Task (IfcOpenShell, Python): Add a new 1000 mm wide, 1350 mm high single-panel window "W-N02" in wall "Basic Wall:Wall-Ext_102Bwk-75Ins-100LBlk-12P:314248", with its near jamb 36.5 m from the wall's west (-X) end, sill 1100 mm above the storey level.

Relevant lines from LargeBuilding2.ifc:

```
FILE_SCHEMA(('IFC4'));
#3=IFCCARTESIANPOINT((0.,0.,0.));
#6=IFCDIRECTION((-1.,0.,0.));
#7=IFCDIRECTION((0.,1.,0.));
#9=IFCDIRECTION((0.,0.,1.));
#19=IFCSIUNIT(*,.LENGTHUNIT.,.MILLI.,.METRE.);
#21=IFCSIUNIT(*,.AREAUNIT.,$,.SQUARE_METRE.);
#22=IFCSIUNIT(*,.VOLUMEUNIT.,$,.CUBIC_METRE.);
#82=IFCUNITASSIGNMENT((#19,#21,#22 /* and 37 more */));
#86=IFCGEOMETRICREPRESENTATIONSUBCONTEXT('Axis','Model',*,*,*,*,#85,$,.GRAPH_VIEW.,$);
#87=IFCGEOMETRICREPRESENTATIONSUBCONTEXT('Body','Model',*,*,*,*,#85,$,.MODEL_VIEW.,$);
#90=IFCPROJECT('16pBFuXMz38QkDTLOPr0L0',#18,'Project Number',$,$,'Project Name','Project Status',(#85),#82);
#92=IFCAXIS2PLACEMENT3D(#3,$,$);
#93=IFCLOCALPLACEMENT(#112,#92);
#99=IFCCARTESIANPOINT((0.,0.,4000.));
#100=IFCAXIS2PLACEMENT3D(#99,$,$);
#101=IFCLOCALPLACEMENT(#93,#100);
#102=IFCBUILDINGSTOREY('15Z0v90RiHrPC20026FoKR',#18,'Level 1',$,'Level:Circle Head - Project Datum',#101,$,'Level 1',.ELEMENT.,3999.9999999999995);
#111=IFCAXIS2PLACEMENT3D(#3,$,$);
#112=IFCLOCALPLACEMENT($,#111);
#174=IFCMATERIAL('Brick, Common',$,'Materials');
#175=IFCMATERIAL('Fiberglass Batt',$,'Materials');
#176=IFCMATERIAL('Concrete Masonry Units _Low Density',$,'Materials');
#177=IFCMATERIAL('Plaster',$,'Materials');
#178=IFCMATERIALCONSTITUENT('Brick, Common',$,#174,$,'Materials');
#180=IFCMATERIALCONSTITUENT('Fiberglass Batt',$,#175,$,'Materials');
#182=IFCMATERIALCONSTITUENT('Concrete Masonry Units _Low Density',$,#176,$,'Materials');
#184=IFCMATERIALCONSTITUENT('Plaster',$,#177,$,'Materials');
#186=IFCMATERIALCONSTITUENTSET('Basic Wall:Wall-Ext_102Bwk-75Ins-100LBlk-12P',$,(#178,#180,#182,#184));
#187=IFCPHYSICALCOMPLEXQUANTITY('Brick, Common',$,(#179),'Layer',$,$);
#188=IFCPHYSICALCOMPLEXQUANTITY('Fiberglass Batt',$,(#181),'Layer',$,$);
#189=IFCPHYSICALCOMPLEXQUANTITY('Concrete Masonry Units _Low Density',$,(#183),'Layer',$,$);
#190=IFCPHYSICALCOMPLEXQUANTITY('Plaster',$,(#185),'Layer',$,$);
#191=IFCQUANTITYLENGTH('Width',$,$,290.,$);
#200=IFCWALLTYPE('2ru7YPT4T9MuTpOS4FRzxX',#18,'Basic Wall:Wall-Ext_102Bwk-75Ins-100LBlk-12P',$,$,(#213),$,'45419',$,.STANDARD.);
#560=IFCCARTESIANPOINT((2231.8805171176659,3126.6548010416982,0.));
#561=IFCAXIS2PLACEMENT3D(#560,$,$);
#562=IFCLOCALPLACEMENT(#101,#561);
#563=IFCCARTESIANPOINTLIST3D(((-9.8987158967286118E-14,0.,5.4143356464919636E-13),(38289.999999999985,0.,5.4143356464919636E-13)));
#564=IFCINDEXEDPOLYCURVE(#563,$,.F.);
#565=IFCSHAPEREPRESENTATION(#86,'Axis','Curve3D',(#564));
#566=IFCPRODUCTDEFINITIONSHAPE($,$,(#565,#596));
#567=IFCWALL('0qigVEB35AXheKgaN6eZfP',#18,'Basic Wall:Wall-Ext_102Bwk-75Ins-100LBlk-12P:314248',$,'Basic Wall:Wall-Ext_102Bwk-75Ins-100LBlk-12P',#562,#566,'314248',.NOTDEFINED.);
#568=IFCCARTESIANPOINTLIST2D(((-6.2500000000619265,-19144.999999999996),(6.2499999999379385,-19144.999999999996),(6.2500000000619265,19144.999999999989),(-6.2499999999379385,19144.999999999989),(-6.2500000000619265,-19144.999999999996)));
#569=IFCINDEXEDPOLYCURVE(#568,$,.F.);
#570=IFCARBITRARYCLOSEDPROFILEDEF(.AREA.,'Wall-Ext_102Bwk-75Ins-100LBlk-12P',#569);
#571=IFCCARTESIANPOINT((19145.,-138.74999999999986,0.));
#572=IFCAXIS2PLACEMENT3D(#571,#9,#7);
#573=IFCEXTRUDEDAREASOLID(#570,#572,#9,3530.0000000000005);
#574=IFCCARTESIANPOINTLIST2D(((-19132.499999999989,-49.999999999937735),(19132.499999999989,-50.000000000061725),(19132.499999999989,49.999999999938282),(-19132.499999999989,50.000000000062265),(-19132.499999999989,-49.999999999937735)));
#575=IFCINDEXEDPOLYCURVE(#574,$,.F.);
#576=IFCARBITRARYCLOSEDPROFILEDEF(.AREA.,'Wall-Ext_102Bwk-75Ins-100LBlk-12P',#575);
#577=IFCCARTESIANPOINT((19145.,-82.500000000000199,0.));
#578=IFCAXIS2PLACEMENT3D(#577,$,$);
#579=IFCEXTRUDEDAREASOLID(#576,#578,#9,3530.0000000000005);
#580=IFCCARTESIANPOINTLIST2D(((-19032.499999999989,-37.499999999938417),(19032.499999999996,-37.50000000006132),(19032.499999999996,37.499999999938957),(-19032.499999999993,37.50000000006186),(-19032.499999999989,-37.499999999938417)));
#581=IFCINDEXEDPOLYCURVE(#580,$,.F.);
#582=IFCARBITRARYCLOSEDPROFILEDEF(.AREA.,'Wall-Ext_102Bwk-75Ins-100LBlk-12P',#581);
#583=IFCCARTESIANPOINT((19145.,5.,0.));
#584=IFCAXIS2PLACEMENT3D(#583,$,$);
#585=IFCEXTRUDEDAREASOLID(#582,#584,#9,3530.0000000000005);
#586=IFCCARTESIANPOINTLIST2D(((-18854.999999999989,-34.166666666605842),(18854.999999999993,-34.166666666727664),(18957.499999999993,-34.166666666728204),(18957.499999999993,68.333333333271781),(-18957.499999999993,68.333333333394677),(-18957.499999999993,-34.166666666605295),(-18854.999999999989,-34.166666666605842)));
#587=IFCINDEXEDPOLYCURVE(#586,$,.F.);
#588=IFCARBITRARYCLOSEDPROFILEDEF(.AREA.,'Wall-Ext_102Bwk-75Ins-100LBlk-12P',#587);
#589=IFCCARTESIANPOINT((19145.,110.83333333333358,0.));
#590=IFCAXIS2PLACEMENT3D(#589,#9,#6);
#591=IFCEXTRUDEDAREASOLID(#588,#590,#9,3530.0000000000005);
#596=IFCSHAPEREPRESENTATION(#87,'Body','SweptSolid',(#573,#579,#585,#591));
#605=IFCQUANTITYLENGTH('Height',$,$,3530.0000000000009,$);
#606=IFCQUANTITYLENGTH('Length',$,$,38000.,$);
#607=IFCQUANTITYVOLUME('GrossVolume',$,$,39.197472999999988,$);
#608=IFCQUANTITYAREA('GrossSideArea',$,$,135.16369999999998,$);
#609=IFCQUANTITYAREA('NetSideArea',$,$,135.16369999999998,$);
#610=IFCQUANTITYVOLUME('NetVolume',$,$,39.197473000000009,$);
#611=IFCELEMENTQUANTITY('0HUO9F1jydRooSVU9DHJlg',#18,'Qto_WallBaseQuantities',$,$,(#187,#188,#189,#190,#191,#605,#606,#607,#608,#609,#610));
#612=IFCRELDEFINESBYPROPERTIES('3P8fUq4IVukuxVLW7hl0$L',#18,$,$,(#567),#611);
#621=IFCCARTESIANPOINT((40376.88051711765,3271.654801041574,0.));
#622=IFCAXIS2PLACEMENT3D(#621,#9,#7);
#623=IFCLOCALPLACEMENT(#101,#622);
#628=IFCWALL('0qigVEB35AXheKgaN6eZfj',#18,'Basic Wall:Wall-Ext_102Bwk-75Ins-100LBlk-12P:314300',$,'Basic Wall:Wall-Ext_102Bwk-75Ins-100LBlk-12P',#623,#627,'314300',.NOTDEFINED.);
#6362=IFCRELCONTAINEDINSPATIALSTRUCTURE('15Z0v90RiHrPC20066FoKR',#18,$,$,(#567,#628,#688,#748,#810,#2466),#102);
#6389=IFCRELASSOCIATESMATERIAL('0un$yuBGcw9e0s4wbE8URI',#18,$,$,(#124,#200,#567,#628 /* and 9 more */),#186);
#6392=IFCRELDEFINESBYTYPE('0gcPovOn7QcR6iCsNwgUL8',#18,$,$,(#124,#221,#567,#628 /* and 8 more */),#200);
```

```python
import numpy as np
import ifcopenshell
import ifcopenshell.api.feature
import ifcopenshell.api.geometry
import ifcopenshell.api.pset
import ifcopenshell.api.root
import ifcopenshell.api.spatial
import ifcopenshell.geom
import ifcopenshell.util.element
import ifcopenshell.util.placement
import ifcopenshell.util.representation
import ifcopenshell.util.shape
import ifcopenshell.util.unit

model = ifcopenshell.open("LargeBuilding2.ifc")
unit_scale = ifcopenshell.util.unit.calculate_unit_scale(model)
area_scale = ifcopenshell.util.unit.calculate_unit_scale(model, "AREAUNIT")
volume_scale = ifcopenshell.util.unit.calculate_unit_scale(model, "VOLUMEUNIT")
settings = ifcopenshell.geom.settings()


def volume(element):
    """Net volume in cubic metres, openings subtracted."""
    shape = ifcopenshell.geom.create_shape(settings, element)
    return ifcopenshell.util.shape.get_volume(shape.geometry)


wall = model.by_id(567)
storey = ifcopenshell.util.element.get_container(wall, ifc_class="IfcBuildingStorey")
context = ifcopenshell.util.representation.get_context(model, "Model", "Body", "MODEL_VIEW")
before = volume(wall)

width, height, from_end, sill = 1, 1.35, 36.5, 1.1  # metres

# The wall runs along its own X axis, and the end named is its -X end.
wall_shape = ifcopenshell.geom.create_shape(settings, wall)
x, y, z = ifcopenshell.util.shape.get_vertices(wall_shape.geometry).T
start = x.min() + from_end
face, thickness = float(y.min()), float(y.max() - y.min())
wall_matrix = ifcopenshell.util.placement.get_local_placement(wall.ObjectPlacement)
level = ifcopenshell.util.placement.get_local_placement(storey.ObjectPlacement)[2, 3]


def in_wall(x, y):
    """Placement at x, y metres in the wall's axes, at sill height."""
    matrix = wall_matrix.copy()
    matrix[:, 3] = wall_matrix @ np.array([x / unit_scale, y / unit_scale, 0.0, 1.0])
    matrix[2, 3] = level + sill / unit_scale
    return matrix


# Opening: a box that overshoots both wall faces by 50 mm.
opening = ifcopenshell.api.root.create_entity(model, ifc_class="IfcOpeningElement", predefined_type="OPENING")
box = ifcopenshell.api.geometry.add_wall_representation(
    model, context=context, length=width, height=height, thickness=thickness + 0.1
)
ifcopenshell.api.geometry.assign_representation(model, product=opening, representation=box)
ifcopenshell.api.geometry.edit_object_placement(model, product=opening, matrix=in_wall(start, face - 0.05), is_si=False)
ifcopenshell.api.feature.add_feature(model, feature=opening, element=wall)

window = ifcopenshell.api.root.create_entity(model, ifc_class="IfcWindow", name="W-N02", predefined_type="WINDOW")
window.OverallWidth, window.OverallHeight = width / unit_scale, height / unit_scale
window.PartitioningType = "SINGLE_PANEL"
body = ifcopenshell.api.geometry.add_window_representation(
    model,
    context=context,
    overall_width=window.OverallWidth,
    overall_height=window.OverallHeight,
    partition_type="SINGLE_PANEL",
)
ifcopenshell.api.geometry.assign_representation(model, product=window, representation=body)
ifcopenshell.api.spatial.assign_container(model, products=[window], relating_structure=storey)
ifcopenshell.api.feature.add_filling(model, opening=opening, element=window)

# Centre the window in the wall's thickness.
ifcopenshell.api.geometry.edit_object_placement(model, product=window, matrix=in_wall(start, face), is_si=False)
window_shape = ifcopenshell.geom.create_shape(settings, window)
depth = ifcopenshell.util.shape.get_vertices(window_shape.geometry)[:, 1]
offset = face + thickness / 2 - (depth.min() + depth.max()) / 2
ifcopenshell.api.geometry.edit_object_placement(model, product=window, matrix=in_wall(start, offset), is_si=False)

after = volume(wall)

# Update the wall's stored quantities.
qto = model.by_id(ifcopenshell.util.element.get_pset(wall, "Qto_WallBaseQuantities", should_inherit=False)["id"])
ifcopenshell.api.pset.edit_qto(model, qto=qto, properties={
    "NetSideArea": after / thickness / area_scale,
    "NetVolume": after / volume_scale,
})

print(f"wall volume {before:.3f} -> {after:.3f} m3")

model.write("LargeBuilding2_v2.ifc")
```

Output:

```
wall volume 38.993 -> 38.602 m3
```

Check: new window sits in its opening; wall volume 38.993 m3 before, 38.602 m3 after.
